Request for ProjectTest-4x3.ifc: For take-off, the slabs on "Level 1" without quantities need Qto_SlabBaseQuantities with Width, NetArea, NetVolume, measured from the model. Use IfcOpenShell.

First a look at what the model holds.

```python
import ifcopenshell
import ifcopenshell.util.element
import ifcopenshell.util.unit

model = ifcopenshell.open("ProjectTest-4x3.ifc")
print(model.schema)
for unit_type in ("LENGTHUNIT", "AREAUNIT", "VOLUMEUNIT"):
    print(unit_type, ifcopenshell.util.unit.calculate_unit_scale(model, unit_type))
storey = next(s for s in model.by_type("IfcBuildingStorey") if s.Name == "Level 1")
slabs = [e for e in ifcopenshell.util.element.get_decomposition(storey) if e.is_a("IfcSlab")]
for e in sorted(slabs, key=lambda e: e.id()):
    print(e.id(), e.is_a(), e.Name, list(ifcopenshell.util.element.get_psets(e, qtos_only=True)), sep=" | ")
```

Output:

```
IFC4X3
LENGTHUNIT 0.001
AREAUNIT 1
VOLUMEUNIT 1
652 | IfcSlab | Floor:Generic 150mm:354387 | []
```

```python
import ifcopenshell
import ifcopenshell.api.pset
import ifcopenshell.geom
import ifcopenshell.util.element
import ifcopenshell.util.shape
import ifcopenshell.util.unit

model = ifcopenshell.open("ProjectTest-4x3.ifc")
unit_scale = ifcopenshell.util.unit.calculate_unit_scale(model)
area_scale = ifcopenshell.util.unit.calculate_unit_scale(model, "AREAUNIT")
volume_scale = ifcopenshell.util.unit.calculate_unit_scale(model, "VOLUMEUNIT")
settings = ifcopenshell.geom.settings()

storey = next(s for s in model.by_type("IfcBuildingStorey") if s.Name == "Level 1")
slabs = [e for e in ifcopenshell.util.element.get_decomposition(storey) if e.is_a("IfcSlab")]

for e in sorted(slabs, key=lambda e: e.id()):
    if ifcopenshell.util.element.get_psets(e, qtos_only=True, should_inherit=False):
        continue
    # Geometry comes back in metres, in the element's own axes.
    shape = ifcopenshell.geom.create_shape(settings, e)
    values = {
        "Width": ifcopenshell.util.shape.get_z(shape.geometry) / unit_scale,
        "NetArea": ifcopenshell.util.shape.get_footprint_area(shape.geometry) / area_scale,
        "NetVolume": ifcopenshell.util.shape.get_volume(shape.geometry) / volume_scale,
    }
    qto = ifcopenshell.api.pset.add_qto(model, product=e, name="Qto_SlabBaseQuantities")
    ifcopenshell.api.pset.edit_qto(model, qto=qto, properties=values)
    print(e.id(), {k: round(v, 3) for k, v in values.items()})

model.write("ProjectTest-4x3_rev.ifc")
```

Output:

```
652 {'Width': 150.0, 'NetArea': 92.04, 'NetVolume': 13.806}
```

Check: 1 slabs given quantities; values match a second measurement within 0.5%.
